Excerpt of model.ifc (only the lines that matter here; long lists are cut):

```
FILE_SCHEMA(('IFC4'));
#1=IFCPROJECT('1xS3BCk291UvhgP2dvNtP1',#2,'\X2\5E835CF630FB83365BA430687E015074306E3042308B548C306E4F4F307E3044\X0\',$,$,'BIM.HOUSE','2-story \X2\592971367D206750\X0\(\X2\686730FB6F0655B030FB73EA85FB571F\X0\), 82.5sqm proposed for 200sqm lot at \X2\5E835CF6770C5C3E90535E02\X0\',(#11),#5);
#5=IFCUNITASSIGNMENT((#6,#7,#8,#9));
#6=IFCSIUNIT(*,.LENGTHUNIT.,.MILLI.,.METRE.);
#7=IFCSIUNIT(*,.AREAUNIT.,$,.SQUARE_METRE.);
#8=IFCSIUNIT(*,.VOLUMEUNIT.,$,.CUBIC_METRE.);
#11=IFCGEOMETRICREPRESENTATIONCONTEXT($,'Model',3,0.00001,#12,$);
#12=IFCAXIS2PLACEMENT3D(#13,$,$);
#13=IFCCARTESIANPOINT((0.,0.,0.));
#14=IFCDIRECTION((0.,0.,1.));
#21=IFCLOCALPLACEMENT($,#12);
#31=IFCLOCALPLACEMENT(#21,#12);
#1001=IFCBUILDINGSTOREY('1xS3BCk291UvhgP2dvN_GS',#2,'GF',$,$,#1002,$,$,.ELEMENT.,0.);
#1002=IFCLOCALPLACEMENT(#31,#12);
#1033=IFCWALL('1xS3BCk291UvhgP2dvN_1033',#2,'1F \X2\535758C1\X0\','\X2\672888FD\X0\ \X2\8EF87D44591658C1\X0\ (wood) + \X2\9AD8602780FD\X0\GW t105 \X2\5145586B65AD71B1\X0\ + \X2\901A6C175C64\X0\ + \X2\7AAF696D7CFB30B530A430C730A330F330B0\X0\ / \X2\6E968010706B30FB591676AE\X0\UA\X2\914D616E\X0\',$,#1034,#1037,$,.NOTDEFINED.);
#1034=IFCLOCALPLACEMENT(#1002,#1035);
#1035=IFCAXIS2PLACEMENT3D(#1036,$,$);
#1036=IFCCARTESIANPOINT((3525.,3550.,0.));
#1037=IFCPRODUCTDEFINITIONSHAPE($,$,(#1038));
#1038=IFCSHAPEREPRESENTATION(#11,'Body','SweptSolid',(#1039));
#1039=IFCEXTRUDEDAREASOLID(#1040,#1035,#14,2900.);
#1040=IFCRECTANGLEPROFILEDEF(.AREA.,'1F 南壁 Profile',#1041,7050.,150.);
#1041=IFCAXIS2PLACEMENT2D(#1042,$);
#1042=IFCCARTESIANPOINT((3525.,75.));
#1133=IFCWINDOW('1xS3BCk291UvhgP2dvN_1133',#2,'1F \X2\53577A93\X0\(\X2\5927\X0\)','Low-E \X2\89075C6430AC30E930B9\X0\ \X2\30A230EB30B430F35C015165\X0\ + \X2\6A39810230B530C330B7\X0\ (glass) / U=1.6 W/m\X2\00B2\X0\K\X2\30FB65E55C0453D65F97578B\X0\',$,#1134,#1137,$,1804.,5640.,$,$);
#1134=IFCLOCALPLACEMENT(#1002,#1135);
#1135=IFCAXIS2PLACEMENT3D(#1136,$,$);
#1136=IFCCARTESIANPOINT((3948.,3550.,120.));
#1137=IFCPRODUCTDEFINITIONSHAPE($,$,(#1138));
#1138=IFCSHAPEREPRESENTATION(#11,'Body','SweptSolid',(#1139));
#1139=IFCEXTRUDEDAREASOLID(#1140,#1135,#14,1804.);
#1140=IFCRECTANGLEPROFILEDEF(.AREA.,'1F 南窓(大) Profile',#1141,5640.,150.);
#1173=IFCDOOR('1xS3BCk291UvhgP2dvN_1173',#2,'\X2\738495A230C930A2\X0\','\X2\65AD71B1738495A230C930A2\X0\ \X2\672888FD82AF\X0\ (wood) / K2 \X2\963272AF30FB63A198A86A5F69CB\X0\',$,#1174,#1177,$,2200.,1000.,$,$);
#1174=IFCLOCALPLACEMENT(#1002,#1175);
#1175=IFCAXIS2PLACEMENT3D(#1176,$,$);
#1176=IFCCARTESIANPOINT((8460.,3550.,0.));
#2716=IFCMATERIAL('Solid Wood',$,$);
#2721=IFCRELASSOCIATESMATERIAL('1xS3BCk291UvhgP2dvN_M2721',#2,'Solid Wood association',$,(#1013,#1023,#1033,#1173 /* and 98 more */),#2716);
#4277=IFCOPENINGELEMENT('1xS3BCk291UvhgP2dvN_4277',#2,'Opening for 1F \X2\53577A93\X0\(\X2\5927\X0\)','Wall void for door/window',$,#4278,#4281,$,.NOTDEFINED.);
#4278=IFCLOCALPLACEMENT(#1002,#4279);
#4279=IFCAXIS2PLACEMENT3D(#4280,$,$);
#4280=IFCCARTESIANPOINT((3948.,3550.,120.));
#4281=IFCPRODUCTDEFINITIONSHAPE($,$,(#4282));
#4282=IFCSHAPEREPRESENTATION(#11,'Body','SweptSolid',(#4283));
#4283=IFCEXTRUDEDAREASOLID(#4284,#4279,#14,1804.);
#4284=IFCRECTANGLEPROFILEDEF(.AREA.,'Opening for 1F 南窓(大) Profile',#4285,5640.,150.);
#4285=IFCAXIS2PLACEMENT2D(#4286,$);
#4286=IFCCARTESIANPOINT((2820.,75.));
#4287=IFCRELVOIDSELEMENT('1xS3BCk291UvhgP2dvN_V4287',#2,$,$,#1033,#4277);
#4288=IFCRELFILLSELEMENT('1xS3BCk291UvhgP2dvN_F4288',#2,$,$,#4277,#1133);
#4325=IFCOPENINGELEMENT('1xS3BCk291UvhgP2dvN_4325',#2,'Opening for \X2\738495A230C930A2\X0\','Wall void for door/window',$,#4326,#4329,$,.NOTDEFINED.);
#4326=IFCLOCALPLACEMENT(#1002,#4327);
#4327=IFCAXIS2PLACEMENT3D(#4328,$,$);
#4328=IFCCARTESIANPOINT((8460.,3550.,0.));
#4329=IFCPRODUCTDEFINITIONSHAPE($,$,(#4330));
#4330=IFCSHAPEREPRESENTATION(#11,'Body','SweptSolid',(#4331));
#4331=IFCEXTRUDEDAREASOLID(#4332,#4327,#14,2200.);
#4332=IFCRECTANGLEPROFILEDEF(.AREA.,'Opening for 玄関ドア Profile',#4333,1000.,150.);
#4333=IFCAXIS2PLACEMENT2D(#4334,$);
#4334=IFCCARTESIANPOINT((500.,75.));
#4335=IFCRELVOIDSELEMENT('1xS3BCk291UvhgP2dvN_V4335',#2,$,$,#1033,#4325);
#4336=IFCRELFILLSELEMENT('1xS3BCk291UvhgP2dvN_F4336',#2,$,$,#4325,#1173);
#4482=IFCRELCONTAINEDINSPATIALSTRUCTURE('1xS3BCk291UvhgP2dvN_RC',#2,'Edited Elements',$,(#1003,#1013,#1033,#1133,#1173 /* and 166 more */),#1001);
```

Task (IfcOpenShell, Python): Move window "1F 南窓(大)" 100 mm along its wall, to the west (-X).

```python
import ifcopenshell
import ifcopenshell.api.geometry
import ifcopenshell.util.placement
import ifcopenshell.util.unit

model = ifcopenshell.open("model.ifc")
unit_scale = ifcopenshell.util.unit.calculate_unit_scale(model)

window = model.by_guid("1xS3BCk291UvhgP2dvN_1133")
opening = window.FillsVoids[0].RelatingOpeningElement
wall = opening.VoidsElements[0].RelatingBuildingElement

wall_matrix = ifcopenshell.util.placement.get_local_placement(wall.ObjectPlacement)
shift = wall_matrix[:3, 0] * -0.1 / unit_scale
before = ifcopenshell.util.placement.get_local_placement(window.ObjectPlacement)[:3, 3].copy()

# The window is not placed relative to its opening, so move both.
for product in (opening, window):
    matrix = ifcopenshell.util.placement.get_local_placement(product.ObjectPlacement)
    matrix[:3, 3] += shift
    ifcopenshell.api.geometry.edit_object_placement(model, product=product, matrix=matrix, is_si=False)

after = ifcopenshell.util.placement.get_local_placement(window.ObjectPlacement)[:3, 3]
print("window moved by", (after - before).round(3) + 0.0)

model.write("model_v2.ifc")
```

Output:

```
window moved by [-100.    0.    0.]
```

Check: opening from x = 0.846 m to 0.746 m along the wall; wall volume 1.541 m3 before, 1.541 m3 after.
